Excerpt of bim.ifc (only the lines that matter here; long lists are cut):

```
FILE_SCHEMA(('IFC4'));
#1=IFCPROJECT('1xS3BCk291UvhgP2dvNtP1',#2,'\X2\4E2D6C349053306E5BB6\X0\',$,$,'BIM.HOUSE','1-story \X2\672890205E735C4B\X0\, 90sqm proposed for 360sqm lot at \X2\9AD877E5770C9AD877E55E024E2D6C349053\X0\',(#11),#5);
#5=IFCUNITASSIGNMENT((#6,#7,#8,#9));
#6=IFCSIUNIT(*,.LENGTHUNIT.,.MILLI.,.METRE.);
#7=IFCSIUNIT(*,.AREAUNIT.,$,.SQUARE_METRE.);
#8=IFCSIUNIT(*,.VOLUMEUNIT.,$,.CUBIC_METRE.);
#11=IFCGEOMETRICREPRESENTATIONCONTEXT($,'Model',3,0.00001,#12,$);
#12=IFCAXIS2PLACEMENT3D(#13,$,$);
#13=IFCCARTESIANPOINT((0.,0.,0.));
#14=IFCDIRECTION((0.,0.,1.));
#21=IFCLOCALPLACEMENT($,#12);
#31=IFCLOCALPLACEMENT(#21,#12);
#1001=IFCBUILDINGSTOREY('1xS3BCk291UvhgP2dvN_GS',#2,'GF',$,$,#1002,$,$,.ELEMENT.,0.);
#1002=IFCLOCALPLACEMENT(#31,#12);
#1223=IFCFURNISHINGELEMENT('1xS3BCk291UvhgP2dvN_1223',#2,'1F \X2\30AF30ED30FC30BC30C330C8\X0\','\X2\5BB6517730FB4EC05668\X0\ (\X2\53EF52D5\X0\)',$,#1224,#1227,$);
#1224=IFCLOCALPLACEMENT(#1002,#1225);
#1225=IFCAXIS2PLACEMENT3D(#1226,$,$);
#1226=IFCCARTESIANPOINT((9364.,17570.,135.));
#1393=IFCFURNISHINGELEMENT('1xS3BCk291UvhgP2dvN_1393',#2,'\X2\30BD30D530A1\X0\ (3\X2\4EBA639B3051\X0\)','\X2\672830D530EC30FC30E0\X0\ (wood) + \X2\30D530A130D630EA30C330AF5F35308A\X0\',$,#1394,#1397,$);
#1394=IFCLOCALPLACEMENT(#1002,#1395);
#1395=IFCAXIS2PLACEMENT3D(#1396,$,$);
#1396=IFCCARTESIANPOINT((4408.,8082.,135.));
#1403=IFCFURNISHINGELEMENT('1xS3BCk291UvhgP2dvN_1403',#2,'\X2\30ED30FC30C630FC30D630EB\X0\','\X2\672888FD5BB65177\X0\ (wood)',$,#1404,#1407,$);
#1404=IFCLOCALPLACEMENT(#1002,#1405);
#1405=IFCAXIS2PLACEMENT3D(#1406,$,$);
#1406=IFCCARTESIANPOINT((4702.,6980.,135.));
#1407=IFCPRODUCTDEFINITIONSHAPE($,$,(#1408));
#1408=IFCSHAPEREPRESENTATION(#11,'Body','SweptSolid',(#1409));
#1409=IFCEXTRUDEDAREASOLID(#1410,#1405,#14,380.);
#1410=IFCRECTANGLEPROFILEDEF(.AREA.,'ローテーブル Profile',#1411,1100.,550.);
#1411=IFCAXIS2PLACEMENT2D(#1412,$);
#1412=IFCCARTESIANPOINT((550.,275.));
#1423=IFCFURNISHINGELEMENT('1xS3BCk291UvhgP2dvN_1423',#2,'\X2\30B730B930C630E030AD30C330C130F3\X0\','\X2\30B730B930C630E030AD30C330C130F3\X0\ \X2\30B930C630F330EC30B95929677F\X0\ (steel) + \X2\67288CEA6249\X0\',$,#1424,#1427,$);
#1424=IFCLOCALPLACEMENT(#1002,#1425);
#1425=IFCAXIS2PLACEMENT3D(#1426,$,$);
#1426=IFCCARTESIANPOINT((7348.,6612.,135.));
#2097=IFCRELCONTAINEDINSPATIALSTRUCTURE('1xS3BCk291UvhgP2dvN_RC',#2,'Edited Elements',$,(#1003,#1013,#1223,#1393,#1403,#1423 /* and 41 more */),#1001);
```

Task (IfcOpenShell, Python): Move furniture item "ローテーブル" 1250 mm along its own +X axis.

```python
import ifcopenshell
import ifcopenshell.api.geometry
import ifcopenshell.util.placement
import ifcopenshell.util.unit

model = ifcopenshell.open("bim.ifc")
unit_scale = ifcopenshell.util.unit.calculate_unit_scale(model)

item = model.by_guid("1xS3BCk291UvhgP2dvN_1403")
matrix = ifcopenshell.util.placement.get_local_placement(item.ObjectPlacement)
matrix[:3, 3] += matrix[:3, 0] * 1.25 / unit_scale
ifcopenshell.api.geometry.edit_object_placement(model, product=item, matrix=matrix, is_si=False)

print(ifcopenshell.util.placement.get_local_placement(item.ObjectPlacement).round(3) + 0.0)

model.write("bim_v2.ifc")
```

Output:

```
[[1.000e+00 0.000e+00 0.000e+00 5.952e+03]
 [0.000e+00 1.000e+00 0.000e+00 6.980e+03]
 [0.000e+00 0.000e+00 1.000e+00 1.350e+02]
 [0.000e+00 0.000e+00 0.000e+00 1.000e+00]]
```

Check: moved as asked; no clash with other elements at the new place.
